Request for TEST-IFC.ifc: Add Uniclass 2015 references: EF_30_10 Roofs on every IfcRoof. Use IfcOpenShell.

First a look at what the model holds.

```python
import ifcopenshell

model = ifcopenshell.open("TEST-IFC.ifc")
print(model.schema)
print("classifications:", [c.Name for c in model.by_type("IfcClassification")])
for ifc_class in ("IfcDoor", "IfcRoof", "IfcStair", "IfcWall", "IfcWindow"):
    print(ifc_class, len(model.by_type(ifc_class)))
```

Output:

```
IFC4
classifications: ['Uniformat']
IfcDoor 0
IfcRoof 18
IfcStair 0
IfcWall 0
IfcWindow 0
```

```python
import ifcopenshell
import ifcopenshell.api.classification

model = ifcopenshell.open("TEST-IFC.ifc")

system = ifcopenshell.api.classification.add_classification(model, classification="Uniclass 2015")

codes = {
    "IfcRoof": ("EF_30_10", "Roofs"),
}
for ifc_class, (code, name) in codes.items():
    products = model.by_type(ifc_class)
    ifcopenshell.api.classification.add_reference(
        model, products=products, classification=system, identification=code, name=name
    )
    print(code, len(products))

model.write("TEST-IFC_edited.ifc")
```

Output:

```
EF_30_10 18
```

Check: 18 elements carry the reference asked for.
